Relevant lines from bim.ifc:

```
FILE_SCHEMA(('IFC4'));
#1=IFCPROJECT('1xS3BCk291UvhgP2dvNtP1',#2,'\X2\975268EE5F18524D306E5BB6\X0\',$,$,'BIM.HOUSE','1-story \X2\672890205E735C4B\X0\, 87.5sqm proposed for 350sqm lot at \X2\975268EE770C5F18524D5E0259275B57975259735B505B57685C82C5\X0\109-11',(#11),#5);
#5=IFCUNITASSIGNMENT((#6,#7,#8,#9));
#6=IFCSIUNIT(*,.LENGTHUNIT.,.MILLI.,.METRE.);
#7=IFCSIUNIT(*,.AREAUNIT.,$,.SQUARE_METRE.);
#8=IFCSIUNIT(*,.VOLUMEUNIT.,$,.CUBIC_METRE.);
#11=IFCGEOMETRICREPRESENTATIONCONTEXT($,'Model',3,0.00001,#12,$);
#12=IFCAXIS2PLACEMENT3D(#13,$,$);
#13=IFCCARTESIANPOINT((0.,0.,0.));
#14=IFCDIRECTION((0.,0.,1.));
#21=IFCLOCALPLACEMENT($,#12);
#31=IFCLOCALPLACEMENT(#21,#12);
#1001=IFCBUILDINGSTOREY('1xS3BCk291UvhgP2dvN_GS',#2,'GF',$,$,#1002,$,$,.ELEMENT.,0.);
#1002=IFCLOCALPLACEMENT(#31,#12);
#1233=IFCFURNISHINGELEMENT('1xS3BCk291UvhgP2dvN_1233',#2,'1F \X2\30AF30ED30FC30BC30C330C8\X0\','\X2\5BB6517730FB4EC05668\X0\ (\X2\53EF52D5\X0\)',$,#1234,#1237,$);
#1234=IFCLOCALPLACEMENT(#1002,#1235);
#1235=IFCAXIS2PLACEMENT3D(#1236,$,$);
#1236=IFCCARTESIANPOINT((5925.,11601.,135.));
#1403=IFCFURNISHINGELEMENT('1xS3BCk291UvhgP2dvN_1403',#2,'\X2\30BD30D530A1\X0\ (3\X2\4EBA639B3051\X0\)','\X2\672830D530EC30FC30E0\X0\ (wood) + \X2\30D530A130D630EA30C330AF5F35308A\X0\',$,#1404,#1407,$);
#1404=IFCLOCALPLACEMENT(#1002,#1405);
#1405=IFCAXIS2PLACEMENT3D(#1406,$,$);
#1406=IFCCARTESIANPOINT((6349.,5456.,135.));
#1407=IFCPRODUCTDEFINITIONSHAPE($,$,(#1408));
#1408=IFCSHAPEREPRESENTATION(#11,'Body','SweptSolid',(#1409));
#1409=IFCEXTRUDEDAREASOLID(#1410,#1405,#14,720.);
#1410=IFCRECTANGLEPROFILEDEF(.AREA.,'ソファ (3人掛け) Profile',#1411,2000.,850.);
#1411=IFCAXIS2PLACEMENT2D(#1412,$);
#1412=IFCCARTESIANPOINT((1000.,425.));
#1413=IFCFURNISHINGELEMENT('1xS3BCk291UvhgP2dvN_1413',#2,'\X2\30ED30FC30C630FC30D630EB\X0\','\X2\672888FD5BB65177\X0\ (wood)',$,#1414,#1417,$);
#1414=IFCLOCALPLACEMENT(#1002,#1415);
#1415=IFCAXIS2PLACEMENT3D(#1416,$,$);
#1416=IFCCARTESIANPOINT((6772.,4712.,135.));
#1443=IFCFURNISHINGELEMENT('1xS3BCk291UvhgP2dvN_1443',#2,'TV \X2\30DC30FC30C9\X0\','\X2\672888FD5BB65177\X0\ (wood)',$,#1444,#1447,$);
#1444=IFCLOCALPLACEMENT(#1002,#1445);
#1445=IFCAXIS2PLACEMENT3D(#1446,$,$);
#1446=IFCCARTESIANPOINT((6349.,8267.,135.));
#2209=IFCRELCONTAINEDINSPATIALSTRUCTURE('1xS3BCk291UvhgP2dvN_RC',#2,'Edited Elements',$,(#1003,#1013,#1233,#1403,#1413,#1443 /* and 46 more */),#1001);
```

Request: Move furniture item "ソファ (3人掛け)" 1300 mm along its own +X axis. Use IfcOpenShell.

```python
import ifcopenshell
import ifcopenshell.api.geometry
import ifcopenshell.util.placement
import ifcopenshell.util.unit

model = ifcopenshell.open("bim.ifc")
unit_scale = ifcopenshell.util.unit.calculate_unit_scale(model)

item = model.by_id(1403)
matrix = ifcopenshell.util.placement.get_local_placement(item.ObjectPlacement)
matrix[:3, 3] += matrix[:3, 0] * 1.3 / unit_scale
ifcopenshell.api.geometry.edit_object_placement(model, product=item, matrix=matrix, is_si=False)

print(ifcopenshell.util.placement.get_local_placement(item.ObjectPlacement).round(3) + 0.0)

model.write("bim_v2.ifc")
```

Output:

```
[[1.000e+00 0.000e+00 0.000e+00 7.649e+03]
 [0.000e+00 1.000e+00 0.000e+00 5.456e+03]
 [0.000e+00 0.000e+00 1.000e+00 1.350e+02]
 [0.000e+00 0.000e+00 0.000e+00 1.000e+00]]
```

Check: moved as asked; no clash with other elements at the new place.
